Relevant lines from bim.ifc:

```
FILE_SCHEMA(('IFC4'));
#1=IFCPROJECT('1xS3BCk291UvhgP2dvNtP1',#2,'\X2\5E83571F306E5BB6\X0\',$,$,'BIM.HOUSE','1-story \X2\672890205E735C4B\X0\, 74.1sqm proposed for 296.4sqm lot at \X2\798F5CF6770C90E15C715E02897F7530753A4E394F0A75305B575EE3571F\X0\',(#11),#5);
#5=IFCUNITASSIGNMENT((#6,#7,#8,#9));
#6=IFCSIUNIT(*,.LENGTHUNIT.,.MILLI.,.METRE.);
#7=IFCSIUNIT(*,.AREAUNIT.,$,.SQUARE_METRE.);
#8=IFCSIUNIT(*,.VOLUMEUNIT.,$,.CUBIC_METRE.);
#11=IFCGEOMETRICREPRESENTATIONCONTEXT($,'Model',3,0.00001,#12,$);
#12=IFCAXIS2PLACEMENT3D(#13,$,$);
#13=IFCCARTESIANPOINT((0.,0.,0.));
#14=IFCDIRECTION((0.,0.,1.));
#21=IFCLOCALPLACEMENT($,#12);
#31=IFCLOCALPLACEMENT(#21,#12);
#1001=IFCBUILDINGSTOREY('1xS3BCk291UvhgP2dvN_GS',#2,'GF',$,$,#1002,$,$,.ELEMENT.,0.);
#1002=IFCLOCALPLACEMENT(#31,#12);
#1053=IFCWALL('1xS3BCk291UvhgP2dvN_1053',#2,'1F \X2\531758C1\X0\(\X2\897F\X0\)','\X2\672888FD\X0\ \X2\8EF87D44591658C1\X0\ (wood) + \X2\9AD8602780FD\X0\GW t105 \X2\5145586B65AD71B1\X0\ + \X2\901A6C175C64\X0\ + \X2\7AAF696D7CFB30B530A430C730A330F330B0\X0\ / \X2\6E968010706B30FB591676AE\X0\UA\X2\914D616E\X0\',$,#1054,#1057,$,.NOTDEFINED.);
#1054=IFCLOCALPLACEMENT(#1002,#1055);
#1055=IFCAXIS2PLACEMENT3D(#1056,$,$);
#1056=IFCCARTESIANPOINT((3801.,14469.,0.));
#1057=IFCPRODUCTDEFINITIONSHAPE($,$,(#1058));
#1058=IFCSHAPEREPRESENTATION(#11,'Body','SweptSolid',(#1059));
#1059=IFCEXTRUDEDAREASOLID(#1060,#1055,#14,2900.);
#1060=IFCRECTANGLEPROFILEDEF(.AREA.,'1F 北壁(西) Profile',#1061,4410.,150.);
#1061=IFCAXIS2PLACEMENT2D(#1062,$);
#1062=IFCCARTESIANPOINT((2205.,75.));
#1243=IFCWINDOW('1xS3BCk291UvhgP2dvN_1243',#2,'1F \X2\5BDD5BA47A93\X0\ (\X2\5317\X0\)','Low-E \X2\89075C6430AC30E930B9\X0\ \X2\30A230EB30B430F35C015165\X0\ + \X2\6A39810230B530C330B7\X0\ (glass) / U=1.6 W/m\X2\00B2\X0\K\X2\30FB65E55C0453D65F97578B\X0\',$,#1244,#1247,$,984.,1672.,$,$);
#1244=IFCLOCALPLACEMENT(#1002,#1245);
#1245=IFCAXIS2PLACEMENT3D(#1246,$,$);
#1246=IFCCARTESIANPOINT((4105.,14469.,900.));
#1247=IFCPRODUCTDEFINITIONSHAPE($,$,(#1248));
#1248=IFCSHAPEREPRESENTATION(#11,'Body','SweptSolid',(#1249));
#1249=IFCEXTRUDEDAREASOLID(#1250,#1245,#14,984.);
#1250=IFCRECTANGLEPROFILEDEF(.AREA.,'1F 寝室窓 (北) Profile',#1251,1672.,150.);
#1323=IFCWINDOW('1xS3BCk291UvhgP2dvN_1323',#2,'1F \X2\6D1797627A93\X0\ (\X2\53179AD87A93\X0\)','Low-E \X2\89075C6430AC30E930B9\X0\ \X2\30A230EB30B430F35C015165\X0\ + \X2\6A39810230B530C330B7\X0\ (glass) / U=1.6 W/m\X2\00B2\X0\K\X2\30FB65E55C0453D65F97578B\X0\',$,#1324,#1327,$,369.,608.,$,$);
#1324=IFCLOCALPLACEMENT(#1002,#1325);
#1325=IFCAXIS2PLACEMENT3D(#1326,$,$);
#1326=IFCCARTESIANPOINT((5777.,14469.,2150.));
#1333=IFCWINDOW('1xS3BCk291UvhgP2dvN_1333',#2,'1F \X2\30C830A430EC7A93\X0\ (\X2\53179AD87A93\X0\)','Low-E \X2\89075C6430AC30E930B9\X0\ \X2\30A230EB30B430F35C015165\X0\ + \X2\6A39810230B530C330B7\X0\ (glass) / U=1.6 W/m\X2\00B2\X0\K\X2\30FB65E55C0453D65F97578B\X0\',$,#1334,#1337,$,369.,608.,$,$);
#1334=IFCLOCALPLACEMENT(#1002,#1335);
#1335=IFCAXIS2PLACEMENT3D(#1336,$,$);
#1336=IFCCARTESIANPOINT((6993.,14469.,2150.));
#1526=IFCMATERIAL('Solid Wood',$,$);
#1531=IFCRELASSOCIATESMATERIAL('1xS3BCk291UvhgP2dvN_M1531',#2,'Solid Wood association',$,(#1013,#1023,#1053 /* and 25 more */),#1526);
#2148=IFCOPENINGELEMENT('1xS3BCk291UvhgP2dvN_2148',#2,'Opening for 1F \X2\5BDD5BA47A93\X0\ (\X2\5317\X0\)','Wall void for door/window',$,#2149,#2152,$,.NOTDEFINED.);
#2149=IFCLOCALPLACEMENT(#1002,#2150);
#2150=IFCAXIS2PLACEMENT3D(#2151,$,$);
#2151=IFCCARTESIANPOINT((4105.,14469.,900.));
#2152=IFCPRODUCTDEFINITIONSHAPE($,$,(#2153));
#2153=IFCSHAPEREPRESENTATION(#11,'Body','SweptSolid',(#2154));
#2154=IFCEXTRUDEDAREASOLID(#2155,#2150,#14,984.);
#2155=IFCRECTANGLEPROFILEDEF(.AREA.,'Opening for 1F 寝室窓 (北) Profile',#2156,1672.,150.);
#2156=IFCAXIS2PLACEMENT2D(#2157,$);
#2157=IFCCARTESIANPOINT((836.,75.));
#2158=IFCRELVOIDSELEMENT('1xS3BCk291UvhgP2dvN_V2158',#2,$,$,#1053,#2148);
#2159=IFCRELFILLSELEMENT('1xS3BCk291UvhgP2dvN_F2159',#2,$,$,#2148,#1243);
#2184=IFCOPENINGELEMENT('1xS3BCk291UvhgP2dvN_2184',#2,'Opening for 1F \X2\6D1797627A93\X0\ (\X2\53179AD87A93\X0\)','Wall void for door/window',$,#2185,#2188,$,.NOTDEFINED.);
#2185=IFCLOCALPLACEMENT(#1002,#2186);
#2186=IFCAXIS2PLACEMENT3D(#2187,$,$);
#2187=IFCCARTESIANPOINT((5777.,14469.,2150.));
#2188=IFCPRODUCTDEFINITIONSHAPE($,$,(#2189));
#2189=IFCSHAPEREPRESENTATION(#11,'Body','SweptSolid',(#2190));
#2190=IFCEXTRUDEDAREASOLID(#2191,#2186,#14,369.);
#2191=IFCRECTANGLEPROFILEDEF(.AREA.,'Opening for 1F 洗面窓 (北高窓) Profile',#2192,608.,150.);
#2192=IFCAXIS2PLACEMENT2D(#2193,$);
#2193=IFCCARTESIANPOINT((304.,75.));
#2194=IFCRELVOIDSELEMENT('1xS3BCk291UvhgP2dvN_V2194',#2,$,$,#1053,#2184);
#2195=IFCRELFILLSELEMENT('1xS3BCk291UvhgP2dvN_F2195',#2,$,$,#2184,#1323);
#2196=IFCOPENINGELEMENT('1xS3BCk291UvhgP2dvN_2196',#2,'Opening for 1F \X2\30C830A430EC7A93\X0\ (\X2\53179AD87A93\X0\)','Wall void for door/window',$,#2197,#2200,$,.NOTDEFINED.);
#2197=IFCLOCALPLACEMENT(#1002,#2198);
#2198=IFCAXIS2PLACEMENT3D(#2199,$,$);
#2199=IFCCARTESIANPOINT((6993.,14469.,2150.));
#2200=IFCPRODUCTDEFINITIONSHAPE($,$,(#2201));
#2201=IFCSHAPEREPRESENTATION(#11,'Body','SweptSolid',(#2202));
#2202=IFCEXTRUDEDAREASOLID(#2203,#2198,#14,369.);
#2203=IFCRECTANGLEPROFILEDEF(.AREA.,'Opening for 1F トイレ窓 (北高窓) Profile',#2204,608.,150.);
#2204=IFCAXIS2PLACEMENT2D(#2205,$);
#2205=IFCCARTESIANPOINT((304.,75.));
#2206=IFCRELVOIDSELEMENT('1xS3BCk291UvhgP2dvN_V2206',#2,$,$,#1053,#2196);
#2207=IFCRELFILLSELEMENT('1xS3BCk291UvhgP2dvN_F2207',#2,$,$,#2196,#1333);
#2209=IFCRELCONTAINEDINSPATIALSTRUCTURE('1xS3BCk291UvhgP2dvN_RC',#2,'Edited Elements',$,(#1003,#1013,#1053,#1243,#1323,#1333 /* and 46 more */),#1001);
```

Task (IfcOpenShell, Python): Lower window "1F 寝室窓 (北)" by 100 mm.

```python
import numpy as np
import ifcopenshell
import ifcopenshell.api.geometry
import ifcopenshell.util.placement
import ifcopenshell.util.unit

model = ifcopenshell.open("bim.ifc")
unit_scale = ifcopenshell.util.unit.calculate_unit_scale(model)

window = model.by_guid("1xS3BCk291UvhgP2dvN_1243")
opening = window.FillsVoids[0].RelatingOpeningElement
dz = -0.1 / unit_scale

shift = np.array([0.0, 0.0, dz])
# The window is not placed relative to its opening, so move both.
for product in (opening, window):
    matrix = ifcopenshell.util.placement.get_local_placement(product.ObjectPlacement)
    matrix[:3, 3] += shift
    ifcopenshell.api.geometry.edit_object_placement(model, product=product, matrix=matrix, is_si=False)

print(f"moved by {dz * unit_scale:+.3f} m")

model.write("bim_rev.ifc")
```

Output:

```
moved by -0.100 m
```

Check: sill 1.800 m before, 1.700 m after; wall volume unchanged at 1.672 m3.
